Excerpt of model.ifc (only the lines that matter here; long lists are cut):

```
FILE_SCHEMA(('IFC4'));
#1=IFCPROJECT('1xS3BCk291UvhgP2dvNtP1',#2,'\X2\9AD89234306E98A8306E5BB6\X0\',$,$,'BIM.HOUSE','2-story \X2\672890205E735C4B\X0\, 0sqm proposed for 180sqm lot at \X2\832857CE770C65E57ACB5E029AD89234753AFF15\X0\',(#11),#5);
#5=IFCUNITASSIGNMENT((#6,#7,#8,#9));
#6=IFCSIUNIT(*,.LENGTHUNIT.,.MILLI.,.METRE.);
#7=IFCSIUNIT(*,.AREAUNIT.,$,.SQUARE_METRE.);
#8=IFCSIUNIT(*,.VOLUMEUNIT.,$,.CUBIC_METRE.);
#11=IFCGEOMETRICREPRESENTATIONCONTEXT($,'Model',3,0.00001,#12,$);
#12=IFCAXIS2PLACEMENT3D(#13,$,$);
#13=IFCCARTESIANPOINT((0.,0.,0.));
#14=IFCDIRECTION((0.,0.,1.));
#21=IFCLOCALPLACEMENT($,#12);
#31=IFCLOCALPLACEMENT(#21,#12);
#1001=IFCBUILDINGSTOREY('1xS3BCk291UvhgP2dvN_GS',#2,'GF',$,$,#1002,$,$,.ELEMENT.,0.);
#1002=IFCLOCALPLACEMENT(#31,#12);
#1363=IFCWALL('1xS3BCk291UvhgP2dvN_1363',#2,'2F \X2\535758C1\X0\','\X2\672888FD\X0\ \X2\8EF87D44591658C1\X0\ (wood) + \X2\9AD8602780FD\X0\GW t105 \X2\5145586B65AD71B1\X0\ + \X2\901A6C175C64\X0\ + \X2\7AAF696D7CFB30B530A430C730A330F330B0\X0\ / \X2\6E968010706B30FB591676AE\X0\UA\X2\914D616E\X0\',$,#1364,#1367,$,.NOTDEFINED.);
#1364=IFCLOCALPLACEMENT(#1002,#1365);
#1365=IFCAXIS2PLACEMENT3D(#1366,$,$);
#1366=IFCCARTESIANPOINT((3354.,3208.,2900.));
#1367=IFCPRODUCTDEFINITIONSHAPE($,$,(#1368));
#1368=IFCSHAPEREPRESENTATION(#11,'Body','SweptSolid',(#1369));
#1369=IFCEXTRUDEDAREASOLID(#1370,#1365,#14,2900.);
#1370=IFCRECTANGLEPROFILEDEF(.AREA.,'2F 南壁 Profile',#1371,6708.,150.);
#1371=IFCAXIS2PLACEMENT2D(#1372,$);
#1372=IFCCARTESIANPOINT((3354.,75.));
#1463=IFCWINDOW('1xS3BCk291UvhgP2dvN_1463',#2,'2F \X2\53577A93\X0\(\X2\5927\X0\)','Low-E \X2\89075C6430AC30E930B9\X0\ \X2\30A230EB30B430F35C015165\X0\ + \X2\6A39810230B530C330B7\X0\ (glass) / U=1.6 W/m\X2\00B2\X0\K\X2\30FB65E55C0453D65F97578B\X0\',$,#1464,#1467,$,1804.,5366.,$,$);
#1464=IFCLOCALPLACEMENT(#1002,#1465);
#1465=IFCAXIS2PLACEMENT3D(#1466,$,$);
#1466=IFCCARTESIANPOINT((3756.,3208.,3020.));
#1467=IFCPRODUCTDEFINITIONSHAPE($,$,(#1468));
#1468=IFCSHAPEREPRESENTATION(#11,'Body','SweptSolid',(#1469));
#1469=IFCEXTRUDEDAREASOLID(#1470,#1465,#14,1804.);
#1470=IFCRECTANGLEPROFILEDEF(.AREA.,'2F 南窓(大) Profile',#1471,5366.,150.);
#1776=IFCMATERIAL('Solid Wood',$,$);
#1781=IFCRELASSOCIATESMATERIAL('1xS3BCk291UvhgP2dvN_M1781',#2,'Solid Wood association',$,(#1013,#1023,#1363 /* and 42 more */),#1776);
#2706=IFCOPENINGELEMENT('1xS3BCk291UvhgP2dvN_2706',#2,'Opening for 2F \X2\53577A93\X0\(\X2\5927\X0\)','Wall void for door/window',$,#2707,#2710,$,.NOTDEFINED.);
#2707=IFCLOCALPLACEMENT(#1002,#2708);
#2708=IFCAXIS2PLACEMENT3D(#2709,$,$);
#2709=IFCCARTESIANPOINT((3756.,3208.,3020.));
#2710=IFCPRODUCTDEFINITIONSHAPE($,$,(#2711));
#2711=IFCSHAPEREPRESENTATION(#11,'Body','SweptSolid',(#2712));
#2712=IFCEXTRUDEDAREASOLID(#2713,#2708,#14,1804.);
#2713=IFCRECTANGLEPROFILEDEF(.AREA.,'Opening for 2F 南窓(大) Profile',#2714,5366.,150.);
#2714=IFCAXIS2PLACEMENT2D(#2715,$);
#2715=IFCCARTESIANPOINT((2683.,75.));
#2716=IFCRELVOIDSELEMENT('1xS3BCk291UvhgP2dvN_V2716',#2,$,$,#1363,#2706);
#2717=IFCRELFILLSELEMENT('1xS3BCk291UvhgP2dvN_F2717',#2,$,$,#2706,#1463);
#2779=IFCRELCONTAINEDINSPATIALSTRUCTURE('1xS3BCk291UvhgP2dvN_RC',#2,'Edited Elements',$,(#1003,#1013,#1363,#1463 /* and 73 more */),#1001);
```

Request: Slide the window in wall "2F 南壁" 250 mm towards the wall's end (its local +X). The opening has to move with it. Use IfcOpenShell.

```python
import ifcopenshell
import ifcopenshell.api.geometry
import ifcopenshell.util.placement
import ifcopenshell.util.unit

model = ifcopenshell.open("model.ifc")
unit_scale = ifcopenshell.util.unit.calculate_unit_scale(model)

window = model.by_guid("1xS3BCk291UvhgP2dvN_1463")
opening = window.FillsVoids[0].RelatingOpeningElement
wall = opening.VoidsElements[0].RelatingBuildingElement

wall_matrix = ifcopenshell.util.placement.get_local_placement(wall.ObjectPlacement)
shift = wall_matrix[:3, 0] * 0.25 / unit_scale
before = ifcopenshell.util.placement.get_local_placement(window.ObjectPlacement)[:3, 3].copy()

# The window is not placed relative to its opening, so move both.
for product in (opening, window):
    matrix = ifcopenshell.util.placement.get_local_placement(product.ObjectPlacement)
    matrix[:3, 3] += shift
    ifcopenshell.api.geometry.edit_object_placement(model, product=product, matrix=matrix, is_si=False)

after = ifcopenshell.util.placement.get_local_placement(window.ObjectPlacement)[:3, 3]
print("window moved by", (after - before).round(3) + 0.0)

model.write("model_edited.ifc")
```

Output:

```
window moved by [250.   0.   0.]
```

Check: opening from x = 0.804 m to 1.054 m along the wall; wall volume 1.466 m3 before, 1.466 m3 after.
